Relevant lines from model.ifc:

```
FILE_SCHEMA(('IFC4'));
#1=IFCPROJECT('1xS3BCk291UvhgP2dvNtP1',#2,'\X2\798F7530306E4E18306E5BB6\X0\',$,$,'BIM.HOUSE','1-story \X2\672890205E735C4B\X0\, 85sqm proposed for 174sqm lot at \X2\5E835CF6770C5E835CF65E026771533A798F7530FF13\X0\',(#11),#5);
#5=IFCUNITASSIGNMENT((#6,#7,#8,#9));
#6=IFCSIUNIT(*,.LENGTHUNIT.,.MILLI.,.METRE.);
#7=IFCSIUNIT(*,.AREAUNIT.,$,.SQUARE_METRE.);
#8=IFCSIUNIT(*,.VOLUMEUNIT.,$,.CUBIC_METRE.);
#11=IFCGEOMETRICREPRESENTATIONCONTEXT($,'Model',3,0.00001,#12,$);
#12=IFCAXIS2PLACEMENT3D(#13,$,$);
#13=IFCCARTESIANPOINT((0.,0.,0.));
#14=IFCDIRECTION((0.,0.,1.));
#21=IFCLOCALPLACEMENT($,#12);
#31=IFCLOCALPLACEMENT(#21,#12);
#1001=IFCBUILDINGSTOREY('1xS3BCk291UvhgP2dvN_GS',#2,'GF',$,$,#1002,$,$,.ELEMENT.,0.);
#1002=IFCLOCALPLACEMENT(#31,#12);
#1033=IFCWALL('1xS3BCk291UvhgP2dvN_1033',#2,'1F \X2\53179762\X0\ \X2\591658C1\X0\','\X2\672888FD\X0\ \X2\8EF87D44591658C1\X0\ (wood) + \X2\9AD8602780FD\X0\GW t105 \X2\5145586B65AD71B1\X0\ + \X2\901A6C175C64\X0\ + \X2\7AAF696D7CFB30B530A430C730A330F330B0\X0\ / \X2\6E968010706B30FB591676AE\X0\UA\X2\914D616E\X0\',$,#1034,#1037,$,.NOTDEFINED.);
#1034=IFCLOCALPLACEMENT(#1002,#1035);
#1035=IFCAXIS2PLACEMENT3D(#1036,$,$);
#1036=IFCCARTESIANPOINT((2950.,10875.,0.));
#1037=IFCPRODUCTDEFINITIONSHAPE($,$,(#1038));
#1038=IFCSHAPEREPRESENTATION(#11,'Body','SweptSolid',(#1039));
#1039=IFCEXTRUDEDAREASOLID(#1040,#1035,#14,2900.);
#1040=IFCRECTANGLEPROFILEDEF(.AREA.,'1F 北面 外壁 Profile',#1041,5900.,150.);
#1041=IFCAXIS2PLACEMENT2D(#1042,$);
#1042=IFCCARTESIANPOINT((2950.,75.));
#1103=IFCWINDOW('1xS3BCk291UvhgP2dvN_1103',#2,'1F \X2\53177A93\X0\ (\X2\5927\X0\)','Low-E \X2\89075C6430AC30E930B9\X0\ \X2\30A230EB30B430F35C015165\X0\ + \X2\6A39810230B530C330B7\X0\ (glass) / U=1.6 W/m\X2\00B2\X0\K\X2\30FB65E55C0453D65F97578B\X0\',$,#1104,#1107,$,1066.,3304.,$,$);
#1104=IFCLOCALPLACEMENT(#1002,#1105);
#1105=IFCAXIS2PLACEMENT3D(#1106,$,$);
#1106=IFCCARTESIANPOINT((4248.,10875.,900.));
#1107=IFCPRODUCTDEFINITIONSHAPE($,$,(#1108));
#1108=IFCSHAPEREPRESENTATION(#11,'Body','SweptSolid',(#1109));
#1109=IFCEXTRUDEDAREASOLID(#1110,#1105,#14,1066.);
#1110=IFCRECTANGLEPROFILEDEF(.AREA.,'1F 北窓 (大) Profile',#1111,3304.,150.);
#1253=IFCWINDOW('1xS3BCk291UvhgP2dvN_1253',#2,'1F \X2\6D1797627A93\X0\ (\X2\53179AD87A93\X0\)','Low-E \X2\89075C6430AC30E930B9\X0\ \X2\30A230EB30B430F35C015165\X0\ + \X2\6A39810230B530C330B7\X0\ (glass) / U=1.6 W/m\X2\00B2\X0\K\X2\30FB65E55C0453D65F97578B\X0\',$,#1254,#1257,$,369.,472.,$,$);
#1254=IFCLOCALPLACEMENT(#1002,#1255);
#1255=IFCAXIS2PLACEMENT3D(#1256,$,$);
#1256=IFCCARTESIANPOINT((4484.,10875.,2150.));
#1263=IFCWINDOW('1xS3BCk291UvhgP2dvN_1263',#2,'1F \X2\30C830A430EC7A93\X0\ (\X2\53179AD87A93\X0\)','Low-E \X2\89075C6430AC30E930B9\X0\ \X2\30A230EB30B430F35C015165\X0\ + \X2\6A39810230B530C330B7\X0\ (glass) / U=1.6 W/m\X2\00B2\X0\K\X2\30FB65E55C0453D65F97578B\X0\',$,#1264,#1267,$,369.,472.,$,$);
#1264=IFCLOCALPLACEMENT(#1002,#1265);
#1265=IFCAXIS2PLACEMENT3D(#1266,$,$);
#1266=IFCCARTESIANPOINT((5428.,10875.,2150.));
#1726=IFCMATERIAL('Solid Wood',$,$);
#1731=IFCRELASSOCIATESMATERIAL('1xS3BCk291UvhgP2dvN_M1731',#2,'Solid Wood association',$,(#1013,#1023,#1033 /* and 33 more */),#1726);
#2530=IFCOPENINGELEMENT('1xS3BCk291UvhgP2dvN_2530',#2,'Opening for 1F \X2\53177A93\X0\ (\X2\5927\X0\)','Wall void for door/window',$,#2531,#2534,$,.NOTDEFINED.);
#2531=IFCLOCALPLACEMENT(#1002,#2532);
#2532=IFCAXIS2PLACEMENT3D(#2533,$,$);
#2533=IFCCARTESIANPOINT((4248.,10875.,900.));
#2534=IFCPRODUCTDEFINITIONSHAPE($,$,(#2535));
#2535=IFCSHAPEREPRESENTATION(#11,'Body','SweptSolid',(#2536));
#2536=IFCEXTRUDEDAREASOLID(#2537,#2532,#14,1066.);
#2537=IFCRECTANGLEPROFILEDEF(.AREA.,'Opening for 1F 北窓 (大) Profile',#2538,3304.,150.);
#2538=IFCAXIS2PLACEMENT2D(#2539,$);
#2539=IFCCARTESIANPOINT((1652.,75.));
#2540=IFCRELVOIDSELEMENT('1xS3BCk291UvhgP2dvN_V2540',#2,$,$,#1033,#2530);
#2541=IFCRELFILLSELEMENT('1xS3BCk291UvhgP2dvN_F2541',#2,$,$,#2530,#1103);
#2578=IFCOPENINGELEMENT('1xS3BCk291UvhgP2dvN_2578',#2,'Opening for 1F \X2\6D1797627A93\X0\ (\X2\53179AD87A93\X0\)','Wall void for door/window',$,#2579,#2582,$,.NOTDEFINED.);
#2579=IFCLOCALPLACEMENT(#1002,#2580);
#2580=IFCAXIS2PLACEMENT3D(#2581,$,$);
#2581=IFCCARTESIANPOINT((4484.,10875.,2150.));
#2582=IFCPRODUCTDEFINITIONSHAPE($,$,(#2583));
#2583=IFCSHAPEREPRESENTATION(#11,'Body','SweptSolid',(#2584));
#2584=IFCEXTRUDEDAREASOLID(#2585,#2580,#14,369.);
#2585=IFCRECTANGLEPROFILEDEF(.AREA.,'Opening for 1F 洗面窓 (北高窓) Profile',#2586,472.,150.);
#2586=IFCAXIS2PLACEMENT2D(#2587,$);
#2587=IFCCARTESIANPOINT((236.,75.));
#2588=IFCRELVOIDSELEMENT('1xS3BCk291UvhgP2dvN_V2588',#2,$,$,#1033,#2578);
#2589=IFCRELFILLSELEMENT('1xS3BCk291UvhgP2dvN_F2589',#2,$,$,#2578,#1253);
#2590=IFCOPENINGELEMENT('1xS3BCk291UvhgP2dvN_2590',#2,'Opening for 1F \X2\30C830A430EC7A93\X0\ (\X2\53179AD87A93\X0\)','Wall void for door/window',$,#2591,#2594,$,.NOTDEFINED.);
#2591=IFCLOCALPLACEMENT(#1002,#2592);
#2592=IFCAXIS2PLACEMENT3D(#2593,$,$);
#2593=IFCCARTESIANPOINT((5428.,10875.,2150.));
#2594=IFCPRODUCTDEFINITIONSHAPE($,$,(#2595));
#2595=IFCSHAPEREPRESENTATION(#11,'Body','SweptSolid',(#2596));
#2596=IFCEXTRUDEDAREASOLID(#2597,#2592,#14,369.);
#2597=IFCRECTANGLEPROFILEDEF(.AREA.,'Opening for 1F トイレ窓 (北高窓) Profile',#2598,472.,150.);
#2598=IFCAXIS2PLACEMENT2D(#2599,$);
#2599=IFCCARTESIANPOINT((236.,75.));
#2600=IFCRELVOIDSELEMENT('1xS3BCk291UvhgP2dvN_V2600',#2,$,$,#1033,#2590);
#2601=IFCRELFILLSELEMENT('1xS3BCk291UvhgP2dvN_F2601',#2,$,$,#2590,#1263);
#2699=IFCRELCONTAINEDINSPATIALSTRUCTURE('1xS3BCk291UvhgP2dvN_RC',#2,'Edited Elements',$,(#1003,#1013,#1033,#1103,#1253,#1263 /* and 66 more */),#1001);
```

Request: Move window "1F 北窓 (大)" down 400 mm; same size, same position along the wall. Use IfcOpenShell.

```python
import numpy as np
import ifcopenshell
import ifcopenshell.api.geometry
import ifcopenshell.util.placement
import ifcopenshell.util.unit

model = ifcopenshell.open("model.ifc")
unit_scale = ifcopenshell.util.unit.calculate_unit_scale(model)

window = model.by_guid("1xS3BCk291UvhgP2dvN_1103")
opening = window.FillsVoids[0].RelatingOpeningElement
dz = -400.0

shift = np.array([0.0, 0.0, dz])
# The window is not placed relative to its opening, so move both.
for product in (opening, window):
    matrix = ifcopenshell.util.placement.get_local_placement(product.ObjectPlacement)
    matrix[:3, 3] += shift
    ifcopenshell.api.geometry.edit_object_placement(model, product=product, matrix=matrix, is_si=False)

print(f"moved by {dz * unit_scale:+.3f} m")

model.write("model-out.ifc")
```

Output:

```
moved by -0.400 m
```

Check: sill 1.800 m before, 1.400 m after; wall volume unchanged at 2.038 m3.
